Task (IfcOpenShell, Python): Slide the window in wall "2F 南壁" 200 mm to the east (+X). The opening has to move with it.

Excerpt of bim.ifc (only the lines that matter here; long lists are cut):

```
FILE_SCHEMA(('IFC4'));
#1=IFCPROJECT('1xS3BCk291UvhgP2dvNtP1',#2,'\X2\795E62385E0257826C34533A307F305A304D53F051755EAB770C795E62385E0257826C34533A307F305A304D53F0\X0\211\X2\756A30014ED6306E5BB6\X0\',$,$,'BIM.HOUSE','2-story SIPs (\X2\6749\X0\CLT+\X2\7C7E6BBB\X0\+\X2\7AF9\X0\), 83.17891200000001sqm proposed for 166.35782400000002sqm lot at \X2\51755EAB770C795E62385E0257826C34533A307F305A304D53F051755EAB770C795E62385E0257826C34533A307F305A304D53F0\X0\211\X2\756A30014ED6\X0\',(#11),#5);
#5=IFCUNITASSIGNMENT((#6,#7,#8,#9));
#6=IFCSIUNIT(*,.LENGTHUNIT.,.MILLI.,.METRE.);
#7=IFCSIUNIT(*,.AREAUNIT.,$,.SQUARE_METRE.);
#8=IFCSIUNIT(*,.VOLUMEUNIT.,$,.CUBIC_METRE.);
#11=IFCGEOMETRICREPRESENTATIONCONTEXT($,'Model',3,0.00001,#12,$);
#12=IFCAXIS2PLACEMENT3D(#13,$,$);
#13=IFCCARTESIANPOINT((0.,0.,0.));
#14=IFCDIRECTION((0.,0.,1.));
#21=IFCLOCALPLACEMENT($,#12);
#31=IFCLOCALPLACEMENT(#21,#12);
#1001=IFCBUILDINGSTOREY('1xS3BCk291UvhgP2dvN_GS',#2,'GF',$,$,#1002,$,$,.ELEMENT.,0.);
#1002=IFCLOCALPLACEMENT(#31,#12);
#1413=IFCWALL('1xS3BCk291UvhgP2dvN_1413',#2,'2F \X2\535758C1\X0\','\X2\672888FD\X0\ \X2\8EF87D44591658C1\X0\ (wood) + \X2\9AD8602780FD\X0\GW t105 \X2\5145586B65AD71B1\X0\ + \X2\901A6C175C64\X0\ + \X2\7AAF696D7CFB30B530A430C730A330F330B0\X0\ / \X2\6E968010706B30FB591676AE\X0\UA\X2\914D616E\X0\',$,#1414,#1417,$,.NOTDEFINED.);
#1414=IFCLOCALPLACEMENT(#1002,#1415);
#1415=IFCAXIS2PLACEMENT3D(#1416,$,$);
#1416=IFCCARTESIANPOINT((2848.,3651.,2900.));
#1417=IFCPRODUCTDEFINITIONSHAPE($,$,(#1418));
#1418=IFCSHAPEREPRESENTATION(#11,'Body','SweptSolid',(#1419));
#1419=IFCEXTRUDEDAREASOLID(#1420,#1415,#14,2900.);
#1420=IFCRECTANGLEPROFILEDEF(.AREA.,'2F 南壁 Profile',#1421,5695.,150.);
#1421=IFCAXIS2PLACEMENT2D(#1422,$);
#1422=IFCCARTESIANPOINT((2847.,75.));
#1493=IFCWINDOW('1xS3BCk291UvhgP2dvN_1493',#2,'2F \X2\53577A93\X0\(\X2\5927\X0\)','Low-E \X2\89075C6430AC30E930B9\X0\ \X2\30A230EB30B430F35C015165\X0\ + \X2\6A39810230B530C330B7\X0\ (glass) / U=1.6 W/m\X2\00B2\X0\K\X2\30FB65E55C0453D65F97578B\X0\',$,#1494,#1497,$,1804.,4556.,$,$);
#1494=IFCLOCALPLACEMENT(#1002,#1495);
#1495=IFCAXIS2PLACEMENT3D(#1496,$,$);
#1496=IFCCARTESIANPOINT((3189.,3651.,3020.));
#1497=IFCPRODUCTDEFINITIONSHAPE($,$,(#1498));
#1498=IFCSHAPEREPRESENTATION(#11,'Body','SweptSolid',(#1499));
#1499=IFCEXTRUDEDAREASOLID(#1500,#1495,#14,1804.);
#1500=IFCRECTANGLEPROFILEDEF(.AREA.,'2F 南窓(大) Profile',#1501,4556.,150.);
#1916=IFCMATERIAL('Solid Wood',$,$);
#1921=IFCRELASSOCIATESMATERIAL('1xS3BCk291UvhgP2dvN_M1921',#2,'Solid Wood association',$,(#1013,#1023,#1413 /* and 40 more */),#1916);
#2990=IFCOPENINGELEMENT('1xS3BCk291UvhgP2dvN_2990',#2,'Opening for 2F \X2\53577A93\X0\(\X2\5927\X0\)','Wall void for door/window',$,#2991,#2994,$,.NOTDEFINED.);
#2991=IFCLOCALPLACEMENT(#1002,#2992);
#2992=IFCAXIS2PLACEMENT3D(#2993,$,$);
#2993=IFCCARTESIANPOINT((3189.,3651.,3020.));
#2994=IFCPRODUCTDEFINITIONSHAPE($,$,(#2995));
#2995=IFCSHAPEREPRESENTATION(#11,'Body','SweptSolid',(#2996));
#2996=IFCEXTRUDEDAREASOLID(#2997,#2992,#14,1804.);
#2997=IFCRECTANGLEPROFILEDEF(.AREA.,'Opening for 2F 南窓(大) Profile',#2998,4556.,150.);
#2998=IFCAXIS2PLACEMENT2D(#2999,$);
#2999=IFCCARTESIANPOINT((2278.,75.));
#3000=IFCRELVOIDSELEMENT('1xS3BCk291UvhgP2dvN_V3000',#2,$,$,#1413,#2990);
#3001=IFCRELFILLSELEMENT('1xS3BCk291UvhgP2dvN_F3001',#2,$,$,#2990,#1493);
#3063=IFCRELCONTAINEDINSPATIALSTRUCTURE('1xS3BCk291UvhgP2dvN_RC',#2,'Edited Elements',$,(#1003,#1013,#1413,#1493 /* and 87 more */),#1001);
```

```python
import ifcopenshell
import ifcopenshell.api.geometry
import ifcopenshell.util.placement

model = ifcopenshell.open("bim.ifc")

window = model.by_guid("1xS3BCk291UvhgP2dvN_1493")
opening = window.FillsVoids[0].RelatingOpeningElement
wall = opening.VoidsElements[0].RelatingBuildingElement

wall_matrix = ifcopenshell.util.placement.get_local_placement(wall.ObjectPlacement)
shift = wall_matrix[:3, 0] * 200.0
before = ifcopenshell.util.placement.get_local_placement(window.ObjectPlacement)[:3, 3].copy()

# The window is not placed relative to its opening, so move both.
for product in (opening, window):
    matrix = ifcopenshell.util.placement.get_local_placement(product.ObjectPlacement)
    matrix[:3, 3] += shift
    ifcopenshell.api.geometry.edit_object_placement(model, product=product, matrix=matrix, is_si=False)

after = ifcopenshell.util.placement.get_local_placement(window.ObjectPlacement)[:3, 3]
print("window moved by", (after - before).round(3) + 0.0)

model.write("bim_v2.ifc")
```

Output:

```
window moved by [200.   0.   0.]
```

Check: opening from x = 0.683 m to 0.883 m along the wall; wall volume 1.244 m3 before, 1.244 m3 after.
